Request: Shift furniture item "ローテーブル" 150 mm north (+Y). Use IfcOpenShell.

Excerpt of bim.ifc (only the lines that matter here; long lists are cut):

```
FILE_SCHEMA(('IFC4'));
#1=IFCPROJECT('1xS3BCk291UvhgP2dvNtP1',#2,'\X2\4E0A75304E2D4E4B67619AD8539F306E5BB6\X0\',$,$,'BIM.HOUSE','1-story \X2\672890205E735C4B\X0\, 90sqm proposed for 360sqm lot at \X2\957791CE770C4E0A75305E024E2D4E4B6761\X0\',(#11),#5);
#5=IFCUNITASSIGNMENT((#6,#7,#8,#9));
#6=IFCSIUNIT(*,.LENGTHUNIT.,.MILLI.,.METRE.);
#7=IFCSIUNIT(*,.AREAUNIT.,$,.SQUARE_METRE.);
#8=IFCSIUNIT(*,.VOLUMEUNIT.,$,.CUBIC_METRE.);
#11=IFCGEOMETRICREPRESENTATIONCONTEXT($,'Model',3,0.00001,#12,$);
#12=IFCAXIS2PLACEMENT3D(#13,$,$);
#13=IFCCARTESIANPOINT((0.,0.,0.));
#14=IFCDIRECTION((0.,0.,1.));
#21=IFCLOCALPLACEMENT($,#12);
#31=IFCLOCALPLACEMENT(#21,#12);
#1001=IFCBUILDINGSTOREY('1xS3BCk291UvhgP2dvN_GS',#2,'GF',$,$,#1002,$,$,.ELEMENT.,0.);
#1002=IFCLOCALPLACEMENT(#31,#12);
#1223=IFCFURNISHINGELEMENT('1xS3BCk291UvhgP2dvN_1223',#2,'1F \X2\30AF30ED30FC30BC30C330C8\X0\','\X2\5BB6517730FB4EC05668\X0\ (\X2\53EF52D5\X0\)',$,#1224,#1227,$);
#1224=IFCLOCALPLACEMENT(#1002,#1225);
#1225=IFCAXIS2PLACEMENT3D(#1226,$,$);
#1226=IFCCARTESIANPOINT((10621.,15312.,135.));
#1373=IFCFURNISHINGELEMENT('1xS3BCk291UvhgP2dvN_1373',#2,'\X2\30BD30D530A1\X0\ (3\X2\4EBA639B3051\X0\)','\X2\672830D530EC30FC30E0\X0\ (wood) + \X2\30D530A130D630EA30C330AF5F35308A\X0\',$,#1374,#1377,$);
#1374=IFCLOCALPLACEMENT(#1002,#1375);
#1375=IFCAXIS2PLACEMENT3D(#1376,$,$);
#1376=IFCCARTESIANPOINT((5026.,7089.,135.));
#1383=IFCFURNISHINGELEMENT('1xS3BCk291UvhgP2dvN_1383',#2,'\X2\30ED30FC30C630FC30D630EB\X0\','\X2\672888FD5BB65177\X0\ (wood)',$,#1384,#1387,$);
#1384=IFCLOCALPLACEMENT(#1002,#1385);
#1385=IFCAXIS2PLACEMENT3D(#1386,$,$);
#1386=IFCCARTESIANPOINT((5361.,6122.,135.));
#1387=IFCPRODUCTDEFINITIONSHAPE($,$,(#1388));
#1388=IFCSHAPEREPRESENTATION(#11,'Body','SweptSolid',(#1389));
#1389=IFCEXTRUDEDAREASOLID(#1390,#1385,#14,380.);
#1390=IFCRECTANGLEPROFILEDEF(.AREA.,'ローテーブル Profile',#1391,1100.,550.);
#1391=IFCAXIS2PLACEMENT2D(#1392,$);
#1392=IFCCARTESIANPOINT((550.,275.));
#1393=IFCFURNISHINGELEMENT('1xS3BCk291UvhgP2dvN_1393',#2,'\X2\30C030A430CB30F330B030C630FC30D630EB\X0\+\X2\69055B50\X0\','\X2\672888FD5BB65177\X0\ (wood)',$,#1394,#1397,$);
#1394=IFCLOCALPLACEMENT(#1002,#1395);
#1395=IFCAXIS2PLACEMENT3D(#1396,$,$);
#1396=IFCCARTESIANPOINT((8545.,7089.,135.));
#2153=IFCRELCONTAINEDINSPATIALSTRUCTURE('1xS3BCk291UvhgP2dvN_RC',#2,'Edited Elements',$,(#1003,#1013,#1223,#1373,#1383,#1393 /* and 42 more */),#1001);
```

```python
import ifcopenshell
import ifcopenshell.api.geometry
import ifcopenshell.util.placement

model = ifcopenshell.open("bim.ifc")

item = model.by_guid("1xS3BCk291UvhgP2dvN_1383")
matrix = ifcopenshell.util.placement.get_local_placement(item.ObjectPlacement)
matrix[1, 3] += 150.0
ifcopenshell.api.geometry.edit_object_placement(model, product=item, matrix=matrix, is_si=False)

print(ifcopenshell.util.placement.get_local_placement(item.ObjectPlacement).round(3) + 0.0)

model.write("bim_updated.ifc")
```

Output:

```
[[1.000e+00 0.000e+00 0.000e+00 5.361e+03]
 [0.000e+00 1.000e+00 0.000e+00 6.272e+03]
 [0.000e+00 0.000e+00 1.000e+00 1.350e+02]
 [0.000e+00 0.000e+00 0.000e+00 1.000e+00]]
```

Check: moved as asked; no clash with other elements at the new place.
